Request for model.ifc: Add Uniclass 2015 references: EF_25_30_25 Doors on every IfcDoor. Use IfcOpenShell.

First a look at what the model holds.

```python
import ifcopenshell

model = ifcopenshell.open("model.ifc")
print(model.schema)
print("classifications:", [c.Name for c in model.by_type("IfcClassification")])
for ifc_class in ("IfcDoor", "IfcRoof", "IfcStair", "IfcWall", "IfcWindow"):
    print(ifc_class, len(model.by_type(ifc_class)))
```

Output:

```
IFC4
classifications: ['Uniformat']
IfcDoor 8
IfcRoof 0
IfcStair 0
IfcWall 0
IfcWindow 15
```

```python
import ifcopenshell
import ifcopenshell.api.classification

model = ifcopenshell.open("model.ifc")

system = ifcopenshell.api.classification.add_classification(model, classification="Uniclass 2015")

codes = {
    "IfcDoor": ("EF_25_30_25", "Doors"),
}
for ifc_class, (code, name) in codes.items():
    products = model.by_type(ifc_class)
    ifcopenshell.api.classification.add_reference(
        model, products=products, classification=system, identification=code, name=name
    )
    print(code, len(products))

model.write("model_edited.ifc")
```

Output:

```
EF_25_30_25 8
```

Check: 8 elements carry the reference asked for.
